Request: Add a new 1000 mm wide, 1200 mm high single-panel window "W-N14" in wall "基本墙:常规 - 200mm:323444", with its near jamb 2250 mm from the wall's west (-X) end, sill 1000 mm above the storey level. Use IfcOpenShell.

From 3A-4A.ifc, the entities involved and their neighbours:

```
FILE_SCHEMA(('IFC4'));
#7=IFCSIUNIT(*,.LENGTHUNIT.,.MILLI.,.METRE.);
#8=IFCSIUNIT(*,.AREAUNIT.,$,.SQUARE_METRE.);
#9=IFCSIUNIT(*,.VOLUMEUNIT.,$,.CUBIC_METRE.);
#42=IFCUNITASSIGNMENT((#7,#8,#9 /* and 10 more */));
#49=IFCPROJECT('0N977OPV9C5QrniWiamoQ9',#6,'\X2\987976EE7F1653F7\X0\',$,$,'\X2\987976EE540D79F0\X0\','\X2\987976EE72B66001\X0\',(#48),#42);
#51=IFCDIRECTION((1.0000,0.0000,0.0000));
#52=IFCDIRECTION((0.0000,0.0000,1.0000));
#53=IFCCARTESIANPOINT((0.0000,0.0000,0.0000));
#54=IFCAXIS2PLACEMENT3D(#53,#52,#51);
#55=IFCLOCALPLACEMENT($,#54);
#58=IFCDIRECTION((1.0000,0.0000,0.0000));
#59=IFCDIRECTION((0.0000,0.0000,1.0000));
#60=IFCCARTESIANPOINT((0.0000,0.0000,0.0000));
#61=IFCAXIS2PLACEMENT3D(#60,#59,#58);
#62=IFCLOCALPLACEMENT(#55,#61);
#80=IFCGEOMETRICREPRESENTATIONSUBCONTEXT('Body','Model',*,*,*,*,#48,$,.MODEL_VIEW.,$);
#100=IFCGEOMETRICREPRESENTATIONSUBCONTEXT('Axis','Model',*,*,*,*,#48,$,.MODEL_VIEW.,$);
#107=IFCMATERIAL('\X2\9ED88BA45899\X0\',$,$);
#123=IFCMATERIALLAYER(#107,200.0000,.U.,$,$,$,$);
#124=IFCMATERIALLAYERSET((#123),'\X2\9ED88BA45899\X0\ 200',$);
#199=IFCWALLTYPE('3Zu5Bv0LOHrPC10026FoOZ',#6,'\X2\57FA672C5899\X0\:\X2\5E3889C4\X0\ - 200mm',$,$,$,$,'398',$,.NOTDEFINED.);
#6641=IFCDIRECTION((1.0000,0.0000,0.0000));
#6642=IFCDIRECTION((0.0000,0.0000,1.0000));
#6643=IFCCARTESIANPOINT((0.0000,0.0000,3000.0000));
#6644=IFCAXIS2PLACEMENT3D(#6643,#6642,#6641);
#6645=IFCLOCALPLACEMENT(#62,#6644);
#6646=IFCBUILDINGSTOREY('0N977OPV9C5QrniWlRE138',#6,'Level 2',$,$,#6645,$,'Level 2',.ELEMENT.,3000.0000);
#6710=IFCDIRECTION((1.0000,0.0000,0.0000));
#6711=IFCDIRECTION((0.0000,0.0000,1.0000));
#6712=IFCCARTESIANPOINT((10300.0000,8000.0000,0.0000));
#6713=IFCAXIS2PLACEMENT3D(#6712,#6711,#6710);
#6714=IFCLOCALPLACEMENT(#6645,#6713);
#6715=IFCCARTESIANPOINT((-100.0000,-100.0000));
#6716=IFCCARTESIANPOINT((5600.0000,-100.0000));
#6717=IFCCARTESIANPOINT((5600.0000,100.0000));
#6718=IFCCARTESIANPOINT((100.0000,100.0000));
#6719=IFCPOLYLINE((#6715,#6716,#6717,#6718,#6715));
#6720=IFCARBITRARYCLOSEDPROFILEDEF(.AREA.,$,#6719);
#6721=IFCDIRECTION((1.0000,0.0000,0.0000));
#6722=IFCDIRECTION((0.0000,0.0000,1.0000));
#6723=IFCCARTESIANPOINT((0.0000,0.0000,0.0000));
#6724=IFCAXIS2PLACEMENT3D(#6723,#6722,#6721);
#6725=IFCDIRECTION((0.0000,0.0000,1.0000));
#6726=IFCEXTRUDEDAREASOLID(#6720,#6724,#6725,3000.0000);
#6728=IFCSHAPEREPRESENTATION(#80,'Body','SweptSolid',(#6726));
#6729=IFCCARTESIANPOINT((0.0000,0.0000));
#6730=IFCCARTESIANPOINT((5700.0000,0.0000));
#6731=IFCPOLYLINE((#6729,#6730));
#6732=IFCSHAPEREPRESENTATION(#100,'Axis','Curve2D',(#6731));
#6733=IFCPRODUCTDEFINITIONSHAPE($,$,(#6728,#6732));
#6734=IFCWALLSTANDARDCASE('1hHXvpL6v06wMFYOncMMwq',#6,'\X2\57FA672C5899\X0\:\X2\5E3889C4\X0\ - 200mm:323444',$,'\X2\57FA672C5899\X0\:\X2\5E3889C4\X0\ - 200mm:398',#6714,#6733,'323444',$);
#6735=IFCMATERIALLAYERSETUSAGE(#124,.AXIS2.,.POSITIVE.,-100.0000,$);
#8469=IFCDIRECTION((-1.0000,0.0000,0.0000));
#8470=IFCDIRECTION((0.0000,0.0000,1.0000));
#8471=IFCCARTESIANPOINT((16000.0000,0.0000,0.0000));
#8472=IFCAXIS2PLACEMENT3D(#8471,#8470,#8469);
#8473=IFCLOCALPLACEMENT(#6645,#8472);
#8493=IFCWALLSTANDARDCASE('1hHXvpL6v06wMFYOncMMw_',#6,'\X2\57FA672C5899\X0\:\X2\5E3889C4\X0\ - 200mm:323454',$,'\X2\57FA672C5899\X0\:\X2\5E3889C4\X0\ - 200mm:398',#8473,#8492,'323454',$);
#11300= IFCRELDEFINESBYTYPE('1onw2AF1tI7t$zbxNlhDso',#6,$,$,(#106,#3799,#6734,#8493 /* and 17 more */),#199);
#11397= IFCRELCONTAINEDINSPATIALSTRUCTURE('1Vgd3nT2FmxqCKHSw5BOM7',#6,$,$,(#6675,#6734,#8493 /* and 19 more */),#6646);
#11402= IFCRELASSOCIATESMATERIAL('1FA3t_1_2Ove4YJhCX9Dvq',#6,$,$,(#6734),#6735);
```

```python
import numpy as np
import ifcopenshell
import ifcopenshell.api.feature
import ifcopenshell.api.geometry
import ifcopenshell.api.root
import ifcopenshell.api.spatial
import ifcopenshell.geom
import ifcopenshell.util.element
import ifcopenshell.util.placement
import ifcopenshell.util.representation
import ifcopenshell.util.shape
import ifcopenshell.util.unit

model = ifcopenshell.open("3A-4A.ifc")
unit_scale = ifcopenshell.util.unit.calculate_unit_scale(model)
settings = ifcopenshell.geom.settings()


def volume(element):
    """Net volume in cubic metres, openings subtracted."""
    shape = ifcopenshell.geom.create_shape(settings, element)
    return ifcopenshell.util.shape.get_volume(shape.geometry)


wall = model.by_id(6734)
storey = ifcopenshell.util.element.get_container(wall, ifc_class="IfcBuildingStorey")
context = ifcopenshell.util.representation.get_context(model, "Model", "Body", "MODEL_VIEW")
before = volume(wall)

width, height, from_end, sill = 1, 1.2, 2.25, 1  # metres

# The wall runs along its own X axis, and the end named is its -X end.
wall_shape = ifcopenshell.geom.create_shape(settings, wall)
x, y, z = ifcopenshell.util.shape.get_vertices(wall_shape.geometry).T
start = x.min() + from_end
face, thickness = float(y.min()), float(y.max() - y.min())
wall_matrix = ifcopenshell.util.placement.get_local_placement(wall.ObjectPlacement)
level = ifcopenshell.util.placement.get_local_placement(storey.ObjectPlacement)[2, 3]


def in_wall(x, y):
    """Placement at x, y metres in the wall's axes, at sill height."""
    matrix = wall_matrix.copy()
    matrix[:, 3] = wall_matrix @ np.array([x / unit_scale, y / unit_scale, 0.0, 1.0])
    matrix[2, 3] = level + sill / unit_scale
    return matrix


# Opening: a box that overshoots both wall faces by 50 mm.
opening = ifcopenshell.api.root.create_entity(model, ifc_class="IfcOpeningElement", predefined_type="OPENING")
box = ifcopenshell.api.geometry.add_wall_representation(
    model, context=context, length=width, height=height, thickness=thickness + 0.1
)
ifcopenshell.api.geometry.assign_representation(model, product=opening, representation=box)
ifcopenshell.api.geometry.edit_object_placement(model, product=opening, matrix=in_wall(start, face - 0.05), is_si=False)
ifcopenshell.api.feature.add_feature(model, feature=opening, element=wall)

window = ifcopenshell.api.root.create_entity(model, ifc_class="IfcWindow", name="W-N14", predefined_type="WINDOW")
window.OverallWidth, window.OverallHeight = width / unit_scale, height / unit_scale
window.PartitioningType = "SINGLE_PANEL"
body = ifcopenshell.api.geometry.add_window_representation(
    model,
    context=context,
    overall_width=window.OverallWidth,
    overall_height=window.OverallHeight,
    partition_type="SINGLE_PANEL",
)
ifcopenshell.api.geometry.assign_representation(model, product=window, representation=body)
ifcopenshell.api.spatial.assign_container(model, products=[window], relating_structure=storey)
ifcopenshell.api.feature.add_filling(model, opening=opening, element=window)

# Centre the window in the wall's thickness.
ifcopenshell.api.geometry.edit_object_placement(model, product=window, matrix=in_wall(start, face), is_si=False)
window_shape = ifcopenshell.geom.create_shape(settings, window)
depth = ifcopenshell.util.shape.get_vertices(window_shape.geometry)[:, 1]
offset = face + thickness / 2 - (depth.min() + depth.max()) / 2
ifcopenshell.api.geometry.edit_object_placement(model, product=window, matrix=in_wall(start, offset), is_si=False)

after = volume(wall)

print(f"wall volume {before:.3f} -> {after:.3f} m3")

model.write("3A-4A_edited.ifc")
```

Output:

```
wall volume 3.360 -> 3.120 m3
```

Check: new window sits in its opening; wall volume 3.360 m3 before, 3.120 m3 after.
